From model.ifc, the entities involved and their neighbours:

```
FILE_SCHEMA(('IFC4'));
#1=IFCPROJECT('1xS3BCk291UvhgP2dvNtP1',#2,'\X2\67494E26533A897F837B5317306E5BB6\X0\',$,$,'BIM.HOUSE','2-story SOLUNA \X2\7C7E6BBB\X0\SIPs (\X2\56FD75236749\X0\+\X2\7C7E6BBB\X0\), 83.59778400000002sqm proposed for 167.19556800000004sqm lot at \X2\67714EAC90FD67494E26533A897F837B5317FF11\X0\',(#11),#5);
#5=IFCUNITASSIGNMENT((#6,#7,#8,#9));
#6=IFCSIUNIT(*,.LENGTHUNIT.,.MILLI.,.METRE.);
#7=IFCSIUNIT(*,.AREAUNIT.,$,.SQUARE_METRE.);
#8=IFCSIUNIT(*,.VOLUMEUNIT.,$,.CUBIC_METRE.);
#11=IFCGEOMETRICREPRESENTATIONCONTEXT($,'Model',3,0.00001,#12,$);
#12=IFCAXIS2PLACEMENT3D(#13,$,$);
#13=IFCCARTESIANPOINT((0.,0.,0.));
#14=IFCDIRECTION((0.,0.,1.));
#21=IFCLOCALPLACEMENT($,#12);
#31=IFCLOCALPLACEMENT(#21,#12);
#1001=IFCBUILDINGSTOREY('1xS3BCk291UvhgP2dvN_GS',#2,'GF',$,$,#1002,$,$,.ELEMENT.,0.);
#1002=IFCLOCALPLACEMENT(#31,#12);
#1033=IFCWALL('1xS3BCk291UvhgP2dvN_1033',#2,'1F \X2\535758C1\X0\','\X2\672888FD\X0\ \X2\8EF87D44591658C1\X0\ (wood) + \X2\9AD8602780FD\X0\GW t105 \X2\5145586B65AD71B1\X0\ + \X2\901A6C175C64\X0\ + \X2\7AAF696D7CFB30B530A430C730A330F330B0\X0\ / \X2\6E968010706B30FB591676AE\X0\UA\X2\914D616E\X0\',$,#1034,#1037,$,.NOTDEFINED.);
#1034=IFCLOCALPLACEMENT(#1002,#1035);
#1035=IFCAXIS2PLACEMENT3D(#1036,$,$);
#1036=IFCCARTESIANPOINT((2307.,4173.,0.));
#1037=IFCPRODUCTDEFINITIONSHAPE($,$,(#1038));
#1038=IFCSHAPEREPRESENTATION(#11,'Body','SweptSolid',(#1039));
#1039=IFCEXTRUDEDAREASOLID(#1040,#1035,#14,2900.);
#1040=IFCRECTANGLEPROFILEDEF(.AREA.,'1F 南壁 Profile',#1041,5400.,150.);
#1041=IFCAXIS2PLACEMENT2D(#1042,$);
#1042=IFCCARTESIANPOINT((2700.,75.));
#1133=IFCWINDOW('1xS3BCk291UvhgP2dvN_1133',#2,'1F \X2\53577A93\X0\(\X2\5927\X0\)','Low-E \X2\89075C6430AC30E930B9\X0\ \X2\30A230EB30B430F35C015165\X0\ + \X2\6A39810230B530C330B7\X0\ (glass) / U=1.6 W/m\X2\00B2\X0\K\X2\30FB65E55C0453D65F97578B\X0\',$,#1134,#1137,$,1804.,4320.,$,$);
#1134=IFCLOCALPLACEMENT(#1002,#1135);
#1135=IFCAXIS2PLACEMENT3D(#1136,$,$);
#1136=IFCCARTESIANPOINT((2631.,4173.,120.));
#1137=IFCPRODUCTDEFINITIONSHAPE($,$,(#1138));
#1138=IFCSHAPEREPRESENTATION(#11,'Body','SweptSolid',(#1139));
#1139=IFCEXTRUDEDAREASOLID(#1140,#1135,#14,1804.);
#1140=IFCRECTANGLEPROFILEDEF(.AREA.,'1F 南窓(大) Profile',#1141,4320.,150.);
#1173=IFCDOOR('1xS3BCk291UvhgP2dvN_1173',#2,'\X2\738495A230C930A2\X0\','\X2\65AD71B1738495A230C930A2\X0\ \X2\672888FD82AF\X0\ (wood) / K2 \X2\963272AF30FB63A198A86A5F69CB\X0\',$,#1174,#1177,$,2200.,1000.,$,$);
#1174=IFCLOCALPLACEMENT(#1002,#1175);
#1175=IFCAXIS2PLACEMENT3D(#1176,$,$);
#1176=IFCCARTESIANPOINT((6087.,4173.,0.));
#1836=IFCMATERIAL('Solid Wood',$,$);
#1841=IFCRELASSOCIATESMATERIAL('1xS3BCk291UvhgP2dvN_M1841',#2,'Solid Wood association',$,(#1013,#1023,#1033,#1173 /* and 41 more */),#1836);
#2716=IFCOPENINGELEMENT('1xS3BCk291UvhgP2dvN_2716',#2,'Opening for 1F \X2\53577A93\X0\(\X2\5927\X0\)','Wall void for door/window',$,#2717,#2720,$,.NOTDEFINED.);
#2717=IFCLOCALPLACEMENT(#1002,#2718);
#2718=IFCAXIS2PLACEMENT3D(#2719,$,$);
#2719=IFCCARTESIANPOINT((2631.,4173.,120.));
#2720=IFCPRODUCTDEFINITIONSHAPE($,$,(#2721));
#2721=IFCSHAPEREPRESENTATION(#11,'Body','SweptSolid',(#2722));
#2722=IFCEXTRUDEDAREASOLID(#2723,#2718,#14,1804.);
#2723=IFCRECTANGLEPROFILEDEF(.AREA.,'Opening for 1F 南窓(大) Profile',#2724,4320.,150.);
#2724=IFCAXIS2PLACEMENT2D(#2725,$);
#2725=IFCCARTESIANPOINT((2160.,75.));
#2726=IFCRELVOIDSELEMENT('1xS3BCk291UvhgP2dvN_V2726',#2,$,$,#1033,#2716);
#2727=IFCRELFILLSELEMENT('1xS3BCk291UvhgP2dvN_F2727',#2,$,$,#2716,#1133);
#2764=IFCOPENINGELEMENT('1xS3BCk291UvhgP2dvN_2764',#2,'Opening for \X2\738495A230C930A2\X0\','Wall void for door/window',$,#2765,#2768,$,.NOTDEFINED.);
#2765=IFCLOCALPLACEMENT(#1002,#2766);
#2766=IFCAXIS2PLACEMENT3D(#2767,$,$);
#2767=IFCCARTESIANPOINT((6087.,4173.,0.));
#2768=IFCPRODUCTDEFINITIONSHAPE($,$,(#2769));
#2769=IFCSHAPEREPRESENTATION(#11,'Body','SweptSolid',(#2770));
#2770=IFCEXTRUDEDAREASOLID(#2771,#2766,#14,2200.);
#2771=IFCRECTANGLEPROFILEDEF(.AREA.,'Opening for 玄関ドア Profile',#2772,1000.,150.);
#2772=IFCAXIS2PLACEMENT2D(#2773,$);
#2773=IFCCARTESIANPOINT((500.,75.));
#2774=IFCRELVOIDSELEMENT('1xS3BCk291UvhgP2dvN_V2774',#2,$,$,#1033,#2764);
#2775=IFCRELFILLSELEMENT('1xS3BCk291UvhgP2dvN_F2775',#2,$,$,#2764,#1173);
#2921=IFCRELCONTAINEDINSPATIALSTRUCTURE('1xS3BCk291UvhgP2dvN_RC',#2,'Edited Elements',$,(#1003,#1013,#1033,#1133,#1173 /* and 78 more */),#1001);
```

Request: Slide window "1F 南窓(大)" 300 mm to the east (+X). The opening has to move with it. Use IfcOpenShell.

```python
import ifcopenshell
import ifcopenshell.api.geometry
import ifcopenshell.util.placement
import ifcopenshell.util.unit

model = ifcopenshell.open("model.ifc")
unit_scale = ifcopenshell.util.unit.calculate_unit_scale(model)

window = model.by_guid("1xS3BCk291UvhgP2dvN_1133")
opening = window.FillsVoids[0].RelatingOpeningElement
wall = opening.VoidsElements[0].RelatingBuildingElement

wall_matrix = ifcopenshell.util.placement.get_local_placement(wall.ObjectPlacement)
shift = wall_matrix[:3, 0] * 0.3 / unit_scale
before = ifcopenshell.util.placement.get_local_placement(window.ObjectPlacement)[:3, 3].copy()

# The window is not placed relative to its opening, so move both.
for product in (opening, window):
    matrix = ifcopenshell.util.placement.get_local_placement(product.ObjectPlacement)
    matrix[:3, 3] += shift
    ifcopenshell.api.geometry.edit_object_placement(model, product=product, matrix=matrix, is_si=False)

after = ifcopenshell.util.placement.get_local_placement(window.ObjectPlacement)[:3, 3]
print("window moved by", (after - before).round(3) + 0.0)

model.write("model-out.ifc")
```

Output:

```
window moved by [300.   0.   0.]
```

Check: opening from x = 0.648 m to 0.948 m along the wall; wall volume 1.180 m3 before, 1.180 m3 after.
